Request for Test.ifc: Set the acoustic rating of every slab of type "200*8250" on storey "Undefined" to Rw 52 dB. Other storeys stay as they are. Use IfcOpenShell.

First a look at what the model holds.

```python
import ifcopenshell
import ifcopenshell.util.element

model = ifcopenshell.open("Test.ifc")
print(model.schema)
storey = next(s for s in model.by_type("IfcBuildingStorey") if s.Name == "Undefined")
slabs = [e for e in ifcopenshell.util.element.get_decomposition(storey) if e.is_a("IfcSlab")]
seen = {}
for e in slabs:
    element_type = ifcopenshell.util.element.get_type(e)
    key = (element_type.Name if element_type != e and element_type else None, ifcopenshell.util.element.get_pset(e, "Pset_SlabCommon", "AcousticRating"))
    seen[key] = seen.get(key, 0) + 1
for (name, value), count in sorted(seen.items(), key=str):
    print(count, "x", name, "|", value)
```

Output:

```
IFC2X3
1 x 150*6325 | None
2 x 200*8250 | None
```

```python
import ifcopenshell
import ifcopenshell.api.pset
import ifcopenshell.util.element

model = ifcopenshell.open("Test.ifc")

storey = next(s for s in model.by_type("IfcBuildingStorey") if s.Name == "Undefined")
slabs = [e for e in ifcopenshell.util.element.get_decomposition(storey) if e.is_a("IfcSlab")]

count = 0
for e in slabs:
    element_type = ifcopenshell.util.element.get_type(e)
    if element_type in (None, e) or element_type.Name != "200*8250":
        continue
    found = ifcopenshell.util.element.get_pset(e, "Pset_SlabCommon", should_inherit=False)
    if found:
        pset = model.by_id(found["id"])
        if len(ifcopenshell.util.element.get_elements_by_pset(pset)) > 1:
            pset = ifcopenshell.api.pset.unshare_pset(model, products=[e], pset=pset)[0]
    else:
        pset = ifcopenshell.api.pset.add_pset(model, product=e, name="Pset_SlabCommon")
    ifcopenshell.api.pset.edit_pset(model, pset=pset, properties={"AcousticRating": "Rw 52 dB"})
    count += 1

print(count, "slabs updated")

model.write("Test_edited.ifc")
```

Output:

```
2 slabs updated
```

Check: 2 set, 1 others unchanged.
